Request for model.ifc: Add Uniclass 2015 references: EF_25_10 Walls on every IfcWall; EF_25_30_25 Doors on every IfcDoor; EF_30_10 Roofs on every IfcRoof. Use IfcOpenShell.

First a look at what the model holds.

```python
import ifcopenshell

model = ifcopenshell.open("model.ifc")
print(model.schema)
print("classifications:", [c.Name for c in model.by_type("IfcClassification")])
for ifc_class in ("IfcDoor", "IfcRoof", "IfcStair", "IfcWall", "IfcWindow"):
    print(ifc_class, len(model.by_type(ifc_class)))
```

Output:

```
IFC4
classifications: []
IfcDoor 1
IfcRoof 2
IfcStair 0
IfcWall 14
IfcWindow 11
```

```python
import ifcopenshell
import ifcopenshell.api.classification

model = ifcopenshell.open("model.ifc")

system = ifcopenshell.api.classification.add_classification(model, classification="Uniclass 2015")

codes = {
    "IfcWall": ("EF_25_10", "Walls"),
    "IfcDoor": ("EF_25_30_25", "Doors"),
    "IfcRoof": ("EF_30_10", "Roofs"),
}
for ifc_class, (code, name) in codes.items():
    products = model.by_type(ifc_class)
    ifcopenshell.api.classification.add_reference(
        model, products=products, classification=system, identification=code, name=name
    )
    print(code, len(products))

model.write("model_edited.ifc")
```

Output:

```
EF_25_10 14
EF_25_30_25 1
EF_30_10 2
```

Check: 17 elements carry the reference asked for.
